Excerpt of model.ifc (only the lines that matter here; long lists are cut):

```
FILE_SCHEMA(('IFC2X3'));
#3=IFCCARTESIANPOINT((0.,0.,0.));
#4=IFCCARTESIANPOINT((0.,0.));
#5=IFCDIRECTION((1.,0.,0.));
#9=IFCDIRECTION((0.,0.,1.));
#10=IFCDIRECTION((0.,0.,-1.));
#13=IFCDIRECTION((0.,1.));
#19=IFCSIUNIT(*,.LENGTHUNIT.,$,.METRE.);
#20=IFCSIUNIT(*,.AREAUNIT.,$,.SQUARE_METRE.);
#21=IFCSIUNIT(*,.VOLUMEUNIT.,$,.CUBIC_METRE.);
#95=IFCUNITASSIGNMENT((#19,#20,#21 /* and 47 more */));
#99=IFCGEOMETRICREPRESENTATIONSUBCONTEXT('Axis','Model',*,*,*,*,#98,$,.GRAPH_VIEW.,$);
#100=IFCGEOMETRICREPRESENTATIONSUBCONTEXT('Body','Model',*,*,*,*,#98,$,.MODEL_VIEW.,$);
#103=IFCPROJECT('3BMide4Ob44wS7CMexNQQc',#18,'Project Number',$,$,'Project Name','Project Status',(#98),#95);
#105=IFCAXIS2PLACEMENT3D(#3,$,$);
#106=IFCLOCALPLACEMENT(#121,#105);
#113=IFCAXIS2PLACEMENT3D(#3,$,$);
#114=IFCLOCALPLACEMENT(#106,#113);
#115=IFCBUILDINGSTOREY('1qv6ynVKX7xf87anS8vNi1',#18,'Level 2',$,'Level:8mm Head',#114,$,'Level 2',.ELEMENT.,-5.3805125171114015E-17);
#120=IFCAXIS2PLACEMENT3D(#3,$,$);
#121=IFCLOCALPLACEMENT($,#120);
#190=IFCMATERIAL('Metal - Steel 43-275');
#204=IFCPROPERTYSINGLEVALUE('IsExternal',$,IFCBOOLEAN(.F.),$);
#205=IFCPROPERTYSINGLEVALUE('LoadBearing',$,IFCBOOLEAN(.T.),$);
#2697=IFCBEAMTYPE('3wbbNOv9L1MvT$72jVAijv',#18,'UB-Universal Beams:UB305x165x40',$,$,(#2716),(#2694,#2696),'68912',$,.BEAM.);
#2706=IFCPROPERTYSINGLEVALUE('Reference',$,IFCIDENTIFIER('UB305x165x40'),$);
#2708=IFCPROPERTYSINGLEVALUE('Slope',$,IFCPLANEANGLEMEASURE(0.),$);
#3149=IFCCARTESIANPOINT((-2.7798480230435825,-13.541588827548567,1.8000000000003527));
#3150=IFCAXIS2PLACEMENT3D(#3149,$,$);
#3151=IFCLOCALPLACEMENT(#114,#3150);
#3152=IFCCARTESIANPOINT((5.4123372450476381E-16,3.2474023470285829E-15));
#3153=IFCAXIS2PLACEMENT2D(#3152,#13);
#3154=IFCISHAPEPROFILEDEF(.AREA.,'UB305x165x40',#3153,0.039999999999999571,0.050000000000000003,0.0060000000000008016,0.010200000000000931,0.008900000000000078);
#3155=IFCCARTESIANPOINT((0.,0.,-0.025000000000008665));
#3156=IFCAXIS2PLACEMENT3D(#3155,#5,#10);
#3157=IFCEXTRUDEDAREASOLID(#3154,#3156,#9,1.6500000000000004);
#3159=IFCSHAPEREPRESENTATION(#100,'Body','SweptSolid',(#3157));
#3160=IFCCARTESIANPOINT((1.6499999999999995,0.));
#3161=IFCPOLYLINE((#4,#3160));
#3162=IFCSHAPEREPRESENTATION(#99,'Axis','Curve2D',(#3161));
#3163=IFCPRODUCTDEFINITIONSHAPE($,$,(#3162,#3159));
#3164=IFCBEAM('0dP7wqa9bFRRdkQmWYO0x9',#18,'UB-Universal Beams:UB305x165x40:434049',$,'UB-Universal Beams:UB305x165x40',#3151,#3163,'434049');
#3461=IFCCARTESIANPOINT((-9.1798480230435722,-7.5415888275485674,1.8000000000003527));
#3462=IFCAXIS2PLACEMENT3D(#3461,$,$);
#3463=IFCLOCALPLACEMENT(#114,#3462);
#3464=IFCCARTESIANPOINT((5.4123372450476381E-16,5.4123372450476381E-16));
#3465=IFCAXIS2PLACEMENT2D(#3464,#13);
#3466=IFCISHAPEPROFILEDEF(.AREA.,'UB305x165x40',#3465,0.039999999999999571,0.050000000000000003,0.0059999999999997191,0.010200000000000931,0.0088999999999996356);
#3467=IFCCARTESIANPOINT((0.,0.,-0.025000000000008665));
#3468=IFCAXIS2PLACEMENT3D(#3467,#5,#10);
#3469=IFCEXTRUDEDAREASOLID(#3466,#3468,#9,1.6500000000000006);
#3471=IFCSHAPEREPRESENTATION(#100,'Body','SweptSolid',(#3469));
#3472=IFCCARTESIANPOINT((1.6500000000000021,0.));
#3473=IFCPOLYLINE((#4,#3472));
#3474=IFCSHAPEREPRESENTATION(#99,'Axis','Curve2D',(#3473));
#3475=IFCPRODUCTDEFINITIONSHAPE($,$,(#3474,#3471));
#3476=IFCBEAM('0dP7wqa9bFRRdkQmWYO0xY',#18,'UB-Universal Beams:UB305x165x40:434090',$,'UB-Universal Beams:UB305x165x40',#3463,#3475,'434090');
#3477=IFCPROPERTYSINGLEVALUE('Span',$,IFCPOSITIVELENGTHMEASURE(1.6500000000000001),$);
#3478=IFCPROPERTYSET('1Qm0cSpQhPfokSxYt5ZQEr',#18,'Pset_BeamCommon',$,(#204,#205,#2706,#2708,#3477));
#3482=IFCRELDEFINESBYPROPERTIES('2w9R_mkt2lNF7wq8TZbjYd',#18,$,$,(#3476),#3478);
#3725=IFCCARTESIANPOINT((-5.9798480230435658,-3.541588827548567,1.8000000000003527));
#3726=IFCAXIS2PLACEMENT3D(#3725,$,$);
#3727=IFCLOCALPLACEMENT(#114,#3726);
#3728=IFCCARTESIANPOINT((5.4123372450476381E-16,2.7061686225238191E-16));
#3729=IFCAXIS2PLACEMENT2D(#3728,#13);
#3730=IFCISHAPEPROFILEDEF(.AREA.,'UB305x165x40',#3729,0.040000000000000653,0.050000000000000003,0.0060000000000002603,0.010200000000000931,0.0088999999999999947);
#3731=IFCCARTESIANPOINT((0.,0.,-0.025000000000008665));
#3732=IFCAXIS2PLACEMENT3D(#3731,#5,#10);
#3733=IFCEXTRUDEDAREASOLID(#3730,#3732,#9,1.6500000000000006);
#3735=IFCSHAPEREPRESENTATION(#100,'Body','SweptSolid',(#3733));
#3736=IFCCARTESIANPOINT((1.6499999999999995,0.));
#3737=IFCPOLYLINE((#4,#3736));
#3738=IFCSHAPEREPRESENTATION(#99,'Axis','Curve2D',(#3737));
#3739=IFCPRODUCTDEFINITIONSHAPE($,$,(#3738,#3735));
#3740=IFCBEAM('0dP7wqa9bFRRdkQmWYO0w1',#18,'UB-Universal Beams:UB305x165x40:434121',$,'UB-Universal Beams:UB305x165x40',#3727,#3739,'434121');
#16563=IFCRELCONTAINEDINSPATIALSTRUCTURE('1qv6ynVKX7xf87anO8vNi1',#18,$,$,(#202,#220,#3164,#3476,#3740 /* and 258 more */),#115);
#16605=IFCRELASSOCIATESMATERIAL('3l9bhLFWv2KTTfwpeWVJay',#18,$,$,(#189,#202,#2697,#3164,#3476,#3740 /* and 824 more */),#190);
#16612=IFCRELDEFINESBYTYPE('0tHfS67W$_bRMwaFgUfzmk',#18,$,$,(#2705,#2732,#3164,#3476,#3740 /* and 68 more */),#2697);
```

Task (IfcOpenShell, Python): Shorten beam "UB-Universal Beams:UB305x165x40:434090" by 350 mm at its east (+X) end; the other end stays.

```python
import numpy as np
import ifcopenshell
import ifcopenshell.api.pset
import ifcopenshell.util.element
import ifcopenshell.util.representation
import ifcopenshell.util.unit

model = ifcopenshell.open("model.ifc")
unit_scale = ifcopenshell.util.unit.calculate_unit_scale(model)

member = model.by_id(3476)
change = -0.35 / unit_scale

# The extrusion runs towards the end named, so only its depth changes.
body = ifcopenshell.util.representation.get_representation(member, "Model", "Body")
solid = body.Items[0]
old_length = solid.Depth
solid.Depth += change

# Move the axis end point with it.
axis = next(r for r in member.Representation.Representations if r.RepresentationIdentifier == "Axis").Items[0]
start, end = (np.array(p.Coordinates) for p in axis.Points)
end = end + (end - start) / np.linalg.norm(end - start) * change
point = model.createIfcCartesianPoint(end.tolist())
axis.Points = [axis.Points[0], point]

# Update the stored length and volume.
pset = model.by_id(ifcopenshell.util.element.get_pset(member, "Pset_BeamCommon", should_inherit=False)["id"])
ifcopenshell.api.pset.edit_pset(model, pset=pset, properties={
    "Span": model.create_entity("IfcPositiveLengthMeasure", solid.Depth),
})

print(f"length {old_length:g} -> {solid.Depth:g}")

model.write("model_rev.ifc")
```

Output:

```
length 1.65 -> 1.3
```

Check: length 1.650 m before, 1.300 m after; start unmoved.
